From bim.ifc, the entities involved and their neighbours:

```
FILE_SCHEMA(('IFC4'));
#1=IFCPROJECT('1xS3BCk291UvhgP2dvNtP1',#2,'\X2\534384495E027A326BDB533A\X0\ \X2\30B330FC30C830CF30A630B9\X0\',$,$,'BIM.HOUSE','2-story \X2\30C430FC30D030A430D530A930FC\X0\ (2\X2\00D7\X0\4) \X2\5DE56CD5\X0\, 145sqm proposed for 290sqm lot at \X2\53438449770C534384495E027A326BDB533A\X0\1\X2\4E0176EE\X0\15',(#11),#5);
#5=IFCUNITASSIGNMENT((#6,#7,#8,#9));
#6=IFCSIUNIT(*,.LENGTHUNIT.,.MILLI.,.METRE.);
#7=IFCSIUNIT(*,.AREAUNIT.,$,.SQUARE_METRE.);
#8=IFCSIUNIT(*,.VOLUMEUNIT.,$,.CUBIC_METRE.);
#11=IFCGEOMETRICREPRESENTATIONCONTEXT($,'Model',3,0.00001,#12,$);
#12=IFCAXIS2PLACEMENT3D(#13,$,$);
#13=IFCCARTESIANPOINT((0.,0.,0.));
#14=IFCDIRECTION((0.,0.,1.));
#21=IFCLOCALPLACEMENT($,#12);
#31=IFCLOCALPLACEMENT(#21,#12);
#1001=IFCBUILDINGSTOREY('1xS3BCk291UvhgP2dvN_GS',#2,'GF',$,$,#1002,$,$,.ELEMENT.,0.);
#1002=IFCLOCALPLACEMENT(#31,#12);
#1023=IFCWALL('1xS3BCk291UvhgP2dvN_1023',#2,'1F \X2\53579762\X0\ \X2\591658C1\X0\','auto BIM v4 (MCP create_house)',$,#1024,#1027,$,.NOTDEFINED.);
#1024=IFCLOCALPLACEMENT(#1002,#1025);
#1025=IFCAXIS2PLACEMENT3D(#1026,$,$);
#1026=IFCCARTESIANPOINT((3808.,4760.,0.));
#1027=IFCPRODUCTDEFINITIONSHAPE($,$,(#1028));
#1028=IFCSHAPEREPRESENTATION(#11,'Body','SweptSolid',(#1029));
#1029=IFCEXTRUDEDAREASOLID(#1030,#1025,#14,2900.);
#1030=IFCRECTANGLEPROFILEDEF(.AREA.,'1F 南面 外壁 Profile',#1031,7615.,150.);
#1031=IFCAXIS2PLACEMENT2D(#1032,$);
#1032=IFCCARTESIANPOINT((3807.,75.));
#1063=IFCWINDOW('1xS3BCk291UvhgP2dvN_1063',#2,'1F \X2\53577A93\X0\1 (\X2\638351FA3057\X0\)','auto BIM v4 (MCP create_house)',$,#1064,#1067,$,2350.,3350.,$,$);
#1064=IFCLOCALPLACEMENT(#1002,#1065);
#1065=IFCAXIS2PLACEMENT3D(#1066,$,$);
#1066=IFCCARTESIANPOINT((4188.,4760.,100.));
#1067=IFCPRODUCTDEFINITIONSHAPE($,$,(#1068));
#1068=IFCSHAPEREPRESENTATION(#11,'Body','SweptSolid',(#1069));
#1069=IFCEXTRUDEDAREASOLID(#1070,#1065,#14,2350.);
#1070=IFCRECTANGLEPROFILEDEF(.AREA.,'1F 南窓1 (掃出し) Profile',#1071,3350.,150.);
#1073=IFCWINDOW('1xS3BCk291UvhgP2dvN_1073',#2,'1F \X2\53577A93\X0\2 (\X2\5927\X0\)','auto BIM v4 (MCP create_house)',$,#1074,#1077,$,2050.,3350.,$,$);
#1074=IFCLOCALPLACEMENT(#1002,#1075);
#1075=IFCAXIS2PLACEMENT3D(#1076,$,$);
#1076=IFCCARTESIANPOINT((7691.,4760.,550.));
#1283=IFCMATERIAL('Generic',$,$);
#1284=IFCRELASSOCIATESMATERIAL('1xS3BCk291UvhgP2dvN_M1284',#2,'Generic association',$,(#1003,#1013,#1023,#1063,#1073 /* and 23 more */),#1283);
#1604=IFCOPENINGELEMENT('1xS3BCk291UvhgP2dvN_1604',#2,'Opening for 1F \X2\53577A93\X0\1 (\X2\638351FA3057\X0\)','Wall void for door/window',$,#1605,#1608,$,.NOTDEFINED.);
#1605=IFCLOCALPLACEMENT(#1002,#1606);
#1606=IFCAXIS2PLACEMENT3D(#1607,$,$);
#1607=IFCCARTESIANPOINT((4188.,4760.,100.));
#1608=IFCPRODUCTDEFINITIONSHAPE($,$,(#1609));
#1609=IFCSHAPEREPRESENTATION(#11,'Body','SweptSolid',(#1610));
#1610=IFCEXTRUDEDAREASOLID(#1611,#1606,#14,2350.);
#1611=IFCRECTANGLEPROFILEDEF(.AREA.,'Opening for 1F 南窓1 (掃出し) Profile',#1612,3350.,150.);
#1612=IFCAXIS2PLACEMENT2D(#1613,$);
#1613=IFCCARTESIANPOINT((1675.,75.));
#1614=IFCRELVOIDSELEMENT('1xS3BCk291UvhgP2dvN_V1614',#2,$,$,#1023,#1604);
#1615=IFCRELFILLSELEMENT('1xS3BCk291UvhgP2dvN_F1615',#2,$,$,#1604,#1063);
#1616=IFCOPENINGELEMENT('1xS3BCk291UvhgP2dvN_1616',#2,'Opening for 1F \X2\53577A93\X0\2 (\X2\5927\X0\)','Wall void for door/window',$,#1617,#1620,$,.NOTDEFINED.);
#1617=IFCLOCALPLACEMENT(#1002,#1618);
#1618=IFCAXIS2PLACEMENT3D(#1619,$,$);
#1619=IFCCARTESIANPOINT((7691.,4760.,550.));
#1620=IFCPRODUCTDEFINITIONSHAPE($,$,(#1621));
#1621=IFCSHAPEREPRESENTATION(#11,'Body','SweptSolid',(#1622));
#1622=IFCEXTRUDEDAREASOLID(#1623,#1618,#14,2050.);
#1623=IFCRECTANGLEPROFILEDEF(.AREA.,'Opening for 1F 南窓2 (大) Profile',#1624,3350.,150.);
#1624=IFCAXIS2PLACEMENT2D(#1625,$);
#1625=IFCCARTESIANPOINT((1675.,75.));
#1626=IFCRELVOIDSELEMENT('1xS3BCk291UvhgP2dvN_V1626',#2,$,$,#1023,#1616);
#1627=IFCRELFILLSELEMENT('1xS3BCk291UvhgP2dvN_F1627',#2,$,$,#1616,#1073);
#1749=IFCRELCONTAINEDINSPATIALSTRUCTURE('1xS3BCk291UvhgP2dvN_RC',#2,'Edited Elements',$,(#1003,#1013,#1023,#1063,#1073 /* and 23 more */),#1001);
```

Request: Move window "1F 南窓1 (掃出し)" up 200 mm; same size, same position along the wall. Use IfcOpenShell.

```python
import numpy as np
import ifcopenshell
import ifcopenshell.api.geometry
import ifcopenshell.util.placement
import ifcopenshell.util.unit

model = ifcopenshell.open("bim.ifc")
unit_scale = ifcopenshell.util.unit.calculate_unit_scale(model)

window = model.by_id(1063)
opening = window.FillsVoids[0].RelatingOpeningElement
dz = 200.0

shift = np.array([0.0, 0.0, dz])
# The window is not placed relative to its opening, so move both.
for product in (opening, window):
    matrix = ifcopenshell.util.placement.get_local_placement(product.ObjectPlacement)
    matrix[:3, 3] += shift
    ifcopenshell.api.geometry.edit_object_placement(model, product=product, matrix=matrix, is_si=False)

print(f"moved by {dz * unit_scale:+.3f} m")

model.write("bim_updated.ifc")
```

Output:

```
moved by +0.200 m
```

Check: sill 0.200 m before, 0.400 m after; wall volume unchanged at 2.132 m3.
